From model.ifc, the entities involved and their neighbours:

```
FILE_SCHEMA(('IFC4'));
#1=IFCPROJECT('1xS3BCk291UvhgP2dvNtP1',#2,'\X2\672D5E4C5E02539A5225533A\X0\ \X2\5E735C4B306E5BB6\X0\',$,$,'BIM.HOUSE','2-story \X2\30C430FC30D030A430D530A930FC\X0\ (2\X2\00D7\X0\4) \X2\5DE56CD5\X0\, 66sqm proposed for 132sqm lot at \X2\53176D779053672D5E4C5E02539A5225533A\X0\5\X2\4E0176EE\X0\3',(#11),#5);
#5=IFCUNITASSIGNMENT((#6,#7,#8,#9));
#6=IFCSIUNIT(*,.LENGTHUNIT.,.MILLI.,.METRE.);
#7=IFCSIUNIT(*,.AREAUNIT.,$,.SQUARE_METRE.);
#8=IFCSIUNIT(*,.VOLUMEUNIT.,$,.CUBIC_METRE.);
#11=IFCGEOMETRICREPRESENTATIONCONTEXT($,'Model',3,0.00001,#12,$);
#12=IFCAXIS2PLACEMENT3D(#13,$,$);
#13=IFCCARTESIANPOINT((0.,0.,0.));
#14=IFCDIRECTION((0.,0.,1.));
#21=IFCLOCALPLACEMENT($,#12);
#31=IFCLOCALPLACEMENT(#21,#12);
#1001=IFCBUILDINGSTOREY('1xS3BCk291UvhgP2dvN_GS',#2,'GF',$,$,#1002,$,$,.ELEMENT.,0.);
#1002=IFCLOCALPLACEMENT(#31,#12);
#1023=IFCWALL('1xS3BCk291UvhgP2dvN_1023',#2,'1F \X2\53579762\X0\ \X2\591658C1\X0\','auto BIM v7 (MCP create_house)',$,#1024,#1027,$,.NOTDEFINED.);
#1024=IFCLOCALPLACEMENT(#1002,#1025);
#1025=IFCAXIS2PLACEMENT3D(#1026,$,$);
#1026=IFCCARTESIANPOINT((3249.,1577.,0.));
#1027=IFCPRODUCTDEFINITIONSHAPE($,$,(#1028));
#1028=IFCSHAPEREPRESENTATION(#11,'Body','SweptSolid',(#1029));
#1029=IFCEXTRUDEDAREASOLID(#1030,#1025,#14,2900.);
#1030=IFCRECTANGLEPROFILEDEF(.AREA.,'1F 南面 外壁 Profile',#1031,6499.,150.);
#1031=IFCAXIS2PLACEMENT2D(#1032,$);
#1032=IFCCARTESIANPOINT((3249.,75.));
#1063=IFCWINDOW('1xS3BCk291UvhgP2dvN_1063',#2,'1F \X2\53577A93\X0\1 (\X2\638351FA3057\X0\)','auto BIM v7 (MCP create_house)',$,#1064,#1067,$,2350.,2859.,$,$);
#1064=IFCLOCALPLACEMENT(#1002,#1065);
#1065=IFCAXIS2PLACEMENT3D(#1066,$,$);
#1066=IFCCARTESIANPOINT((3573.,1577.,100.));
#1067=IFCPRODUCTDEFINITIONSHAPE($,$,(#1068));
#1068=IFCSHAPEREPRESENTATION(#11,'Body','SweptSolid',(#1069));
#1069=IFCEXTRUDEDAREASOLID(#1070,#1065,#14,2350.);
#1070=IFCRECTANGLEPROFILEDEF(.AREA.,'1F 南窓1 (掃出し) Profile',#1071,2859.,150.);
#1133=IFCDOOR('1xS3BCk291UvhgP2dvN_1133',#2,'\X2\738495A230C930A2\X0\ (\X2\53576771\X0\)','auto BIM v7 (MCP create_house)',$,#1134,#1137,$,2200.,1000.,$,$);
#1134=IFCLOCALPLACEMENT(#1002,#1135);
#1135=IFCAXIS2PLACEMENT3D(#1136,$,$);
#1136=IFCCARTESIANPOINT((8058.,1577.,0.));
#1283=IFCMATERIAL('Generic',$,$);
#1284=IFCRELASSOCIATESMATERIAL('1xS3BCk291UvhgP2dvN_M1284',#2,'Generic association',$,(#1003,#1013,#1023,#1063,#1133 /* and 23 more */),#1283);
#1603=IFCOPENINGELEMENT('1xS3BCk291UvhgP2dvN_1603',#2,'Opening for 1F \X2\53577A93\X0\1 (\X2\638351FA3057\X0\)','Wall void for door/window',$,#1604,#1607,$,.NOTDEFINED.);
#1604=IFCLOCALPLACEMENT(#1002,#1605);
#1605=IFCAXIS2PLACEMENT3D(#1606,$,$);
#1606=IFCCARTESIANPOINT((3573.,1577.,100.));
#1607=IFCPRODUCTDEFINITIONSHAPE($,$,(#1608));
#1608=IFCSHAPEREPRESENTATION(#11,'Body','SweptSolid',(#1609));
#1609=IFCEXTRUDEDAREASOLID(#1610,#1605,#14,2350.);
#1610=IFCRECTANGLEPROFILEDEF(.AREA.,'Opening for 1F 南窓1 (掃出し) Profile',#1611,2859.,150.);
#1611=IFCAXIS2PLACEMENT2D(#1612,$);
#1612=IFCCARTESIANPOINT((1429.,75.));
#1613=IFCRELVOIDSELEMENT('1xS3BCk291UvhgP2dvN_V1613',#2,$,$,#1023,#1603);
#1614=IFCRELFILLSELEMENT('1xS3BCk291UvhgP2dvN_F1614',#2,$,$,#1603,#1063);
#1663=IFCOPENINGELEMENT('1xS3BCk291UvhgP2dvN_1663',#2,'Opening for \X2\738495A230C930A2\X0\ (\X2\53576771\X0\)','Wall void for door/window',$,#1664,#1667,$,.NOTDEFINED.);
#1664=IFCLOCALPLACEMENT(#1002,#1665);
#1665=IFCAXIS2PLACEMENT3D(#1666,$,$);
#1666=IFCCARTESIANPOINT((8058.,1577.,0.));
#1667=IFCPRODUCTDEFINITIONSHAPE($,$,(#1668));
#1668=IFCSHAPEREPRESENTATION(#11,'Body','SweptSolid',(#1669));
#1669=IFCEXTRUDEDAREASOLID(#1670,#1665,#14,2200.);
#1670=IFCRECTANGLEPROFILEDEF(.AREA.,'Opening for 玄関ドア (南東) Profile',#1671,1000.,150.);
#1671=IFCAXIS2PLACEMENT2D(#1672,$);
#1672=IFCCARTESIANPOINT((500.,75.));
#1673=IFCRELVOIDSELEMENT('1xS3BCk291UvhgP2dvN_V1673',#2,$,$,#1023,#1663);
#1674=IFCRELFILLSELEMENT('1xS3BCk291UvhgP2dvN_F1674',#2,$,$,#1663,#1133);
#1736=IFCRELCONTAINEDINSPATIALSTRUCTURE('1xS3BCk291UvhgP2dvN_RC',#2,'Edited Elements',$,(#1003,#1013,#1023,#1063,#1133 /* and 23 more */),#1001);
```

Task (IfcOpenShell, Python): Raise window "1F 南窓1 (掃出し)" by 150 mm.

```python
import numpy as np
import ifcopenshell
import ifcopenshell.api.geometry
import ifcopenshell.util.placement
import ifcopenshell.util.unit

model = ifcopenshell.open("model.ifc")
unit_scale = ifcopenshell.util.unit.calculate_unit_scale(model)

window = model.by_id(1063)
opening = window.FillsVoids[0].RelatingOpeningElement
dz = 0.15 / unit_scale

shift = np.array([0.0, 0.0, dz])
# The window is not placed relative to its opening, so move both.
for product in (opening, window):
    matrix = ifcopenshell.util.placement.get_local_placement(product.ObjectPlacement)
    matrix[:3, 3] += shift
    ifcopenshell.api.geometry.edit_object_placement(model, product=product, matrix=matrix, is_si=False)

print(f"moved by {dz * unit_scale:+.3f} m")

model.write("model_rev.ifc")
```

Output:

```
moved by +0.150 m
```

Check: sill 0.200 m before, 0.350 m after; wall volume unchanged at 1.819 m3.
